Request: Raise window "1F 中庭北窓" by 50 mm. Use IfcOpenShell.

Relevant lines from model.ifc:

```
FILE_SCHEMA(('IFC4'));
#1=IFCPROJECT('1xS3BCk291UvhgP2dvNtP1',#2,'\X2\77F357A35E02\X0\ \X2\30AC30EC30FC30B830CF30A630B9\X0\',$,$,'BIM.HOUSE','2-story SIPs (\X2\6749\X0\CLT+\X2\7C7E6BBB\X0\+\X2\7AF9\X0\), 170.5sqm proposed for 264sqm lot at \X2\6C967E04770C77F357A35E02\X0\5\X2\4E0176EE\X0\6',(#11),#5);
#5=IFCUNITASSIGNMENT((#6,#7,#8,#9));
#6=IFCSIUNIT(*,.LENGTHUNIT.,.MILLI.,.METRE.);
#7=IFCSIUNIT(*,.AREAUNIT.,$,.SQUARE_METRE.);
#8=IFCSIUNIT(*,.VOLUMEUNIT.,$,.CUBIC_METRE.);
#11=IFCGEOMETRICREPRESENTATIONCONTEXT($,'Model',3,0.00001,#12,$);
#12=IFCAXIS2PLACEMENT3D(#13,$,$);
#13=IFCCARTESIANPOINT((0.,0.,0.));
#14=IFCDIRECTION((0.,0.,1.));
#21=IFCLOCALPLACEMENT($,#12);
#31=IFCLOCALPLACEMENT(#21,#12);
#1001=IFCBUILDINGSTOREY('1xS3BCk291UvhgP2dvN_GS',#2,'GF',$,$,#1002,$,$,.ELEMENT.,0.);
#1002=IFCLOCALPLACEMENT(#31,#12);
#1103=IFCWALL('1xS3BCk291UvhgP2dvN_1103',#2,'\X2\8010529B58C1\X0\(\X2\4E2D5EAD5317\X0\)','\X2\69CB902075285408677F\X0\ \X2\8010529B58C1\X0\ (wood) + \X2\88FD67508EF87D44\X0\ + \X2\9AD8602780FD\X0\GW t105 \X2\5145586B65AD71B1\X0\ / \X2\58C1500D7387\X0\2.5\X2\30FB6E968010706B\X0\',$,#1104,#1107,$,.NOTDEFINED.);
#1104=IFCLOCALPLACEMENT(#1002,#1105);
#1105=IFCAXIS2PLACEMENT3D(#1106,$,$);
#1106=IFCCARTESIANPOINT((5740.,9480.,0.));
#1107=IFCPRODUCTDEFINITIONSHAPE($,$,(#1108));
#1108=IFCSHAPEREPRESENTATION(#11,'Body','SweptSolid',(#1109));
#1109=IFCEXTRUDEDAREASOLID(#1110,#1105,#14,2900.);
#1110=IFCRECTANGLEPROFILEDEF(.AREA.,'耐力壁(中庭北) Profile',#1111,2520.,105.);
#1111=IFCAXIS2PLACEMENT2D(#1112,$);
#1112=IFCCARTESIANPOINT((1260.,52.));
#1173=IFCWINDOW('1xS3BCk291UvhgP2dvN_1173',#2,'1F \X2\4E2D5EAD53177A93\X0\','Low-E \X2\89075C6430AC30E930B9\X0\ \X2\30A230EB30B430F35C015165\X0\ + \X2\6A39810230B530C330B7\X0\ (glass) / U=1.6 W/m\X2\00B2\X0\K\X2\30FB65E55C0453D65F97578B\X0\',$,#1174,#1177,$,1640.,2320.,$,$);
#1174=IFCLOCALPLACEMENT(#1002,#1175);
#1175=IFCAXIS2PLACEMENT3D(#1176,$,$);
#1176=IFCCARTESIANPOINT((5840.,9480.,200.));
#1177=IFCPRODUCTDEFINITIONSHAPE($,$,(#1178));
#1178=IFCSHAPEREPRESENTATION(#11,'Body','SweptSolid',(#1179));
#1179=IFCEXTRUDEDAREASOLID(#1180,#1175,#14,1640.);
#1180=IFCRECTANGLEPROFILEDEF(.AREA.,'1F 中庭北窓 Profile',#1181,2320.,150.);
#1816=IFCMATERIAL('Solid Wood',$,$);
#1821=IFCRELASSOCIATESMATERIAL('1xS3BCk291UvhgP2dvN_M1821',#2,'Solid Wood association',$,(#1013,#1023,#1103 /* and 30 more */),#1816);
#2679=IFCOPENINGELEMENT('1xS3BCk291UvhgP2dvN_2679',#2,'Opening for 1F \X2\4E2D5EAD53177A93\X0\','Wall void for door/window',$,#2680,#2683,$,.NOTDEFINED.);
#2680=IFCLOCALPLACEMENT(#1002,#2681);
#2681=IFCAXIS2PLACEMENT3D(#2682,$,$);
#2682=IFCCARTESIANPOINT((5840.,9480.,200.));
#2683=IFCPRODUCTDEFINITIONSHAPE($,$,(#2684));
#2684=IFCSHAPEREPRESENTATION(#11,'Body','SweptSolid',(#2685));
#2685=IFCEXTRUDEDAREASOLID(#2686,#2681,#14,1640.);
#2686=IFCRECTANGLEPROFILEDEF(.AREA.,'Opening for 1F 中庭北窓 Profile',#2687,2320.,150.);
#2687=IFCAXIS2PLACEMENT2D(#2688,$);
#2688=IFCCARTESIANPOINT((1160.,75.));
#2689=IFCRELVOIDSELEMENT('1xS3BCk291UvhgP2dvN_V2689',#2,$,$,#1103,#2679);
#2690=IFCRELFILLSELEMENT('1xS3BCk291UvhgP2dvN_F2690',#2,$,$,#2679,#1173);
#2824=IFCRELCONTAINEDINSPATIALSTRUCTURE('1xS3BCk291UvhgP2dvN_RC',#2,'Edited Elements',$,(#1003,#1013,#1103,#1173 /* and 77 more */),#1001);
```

```python
import numpy as np
import ifcopenshell
import ifcopenshell.api.geometry
import ifcopenshell.util.placement
import ifcopenshell.util.unit

model = ifcopenshell.open("model.ifc")
unit_scale = ifcopenshell.util.unit.calculate_unit_scale(model)

window = model.by_guid("1xS3BCk291UvhgP2dvN_1173")
opening = window.FillsVoids[0].RelatingOpeningElement
dz = 0.05 / unit_scale

shift = np.array([0.0, 0.0, dz])
# The window is not placed relative to its opening, so move both.
for product in (opening, window):
    matrix = ifcopenshell.util.placement.get_local_placement(product.ObjectPlacement)
    matrix[:3, 3] += shift
    ifcopenshell.api.geometry.edit_object_placement(model, product=product, matrix=matrix, is_si=False)

print(f"moved by {dz * unit_scale:+.3f} m")

model.write("model_rev.ifc")
```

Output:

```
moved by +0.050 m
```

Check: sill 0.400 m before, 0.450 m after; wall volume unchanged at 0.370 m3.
